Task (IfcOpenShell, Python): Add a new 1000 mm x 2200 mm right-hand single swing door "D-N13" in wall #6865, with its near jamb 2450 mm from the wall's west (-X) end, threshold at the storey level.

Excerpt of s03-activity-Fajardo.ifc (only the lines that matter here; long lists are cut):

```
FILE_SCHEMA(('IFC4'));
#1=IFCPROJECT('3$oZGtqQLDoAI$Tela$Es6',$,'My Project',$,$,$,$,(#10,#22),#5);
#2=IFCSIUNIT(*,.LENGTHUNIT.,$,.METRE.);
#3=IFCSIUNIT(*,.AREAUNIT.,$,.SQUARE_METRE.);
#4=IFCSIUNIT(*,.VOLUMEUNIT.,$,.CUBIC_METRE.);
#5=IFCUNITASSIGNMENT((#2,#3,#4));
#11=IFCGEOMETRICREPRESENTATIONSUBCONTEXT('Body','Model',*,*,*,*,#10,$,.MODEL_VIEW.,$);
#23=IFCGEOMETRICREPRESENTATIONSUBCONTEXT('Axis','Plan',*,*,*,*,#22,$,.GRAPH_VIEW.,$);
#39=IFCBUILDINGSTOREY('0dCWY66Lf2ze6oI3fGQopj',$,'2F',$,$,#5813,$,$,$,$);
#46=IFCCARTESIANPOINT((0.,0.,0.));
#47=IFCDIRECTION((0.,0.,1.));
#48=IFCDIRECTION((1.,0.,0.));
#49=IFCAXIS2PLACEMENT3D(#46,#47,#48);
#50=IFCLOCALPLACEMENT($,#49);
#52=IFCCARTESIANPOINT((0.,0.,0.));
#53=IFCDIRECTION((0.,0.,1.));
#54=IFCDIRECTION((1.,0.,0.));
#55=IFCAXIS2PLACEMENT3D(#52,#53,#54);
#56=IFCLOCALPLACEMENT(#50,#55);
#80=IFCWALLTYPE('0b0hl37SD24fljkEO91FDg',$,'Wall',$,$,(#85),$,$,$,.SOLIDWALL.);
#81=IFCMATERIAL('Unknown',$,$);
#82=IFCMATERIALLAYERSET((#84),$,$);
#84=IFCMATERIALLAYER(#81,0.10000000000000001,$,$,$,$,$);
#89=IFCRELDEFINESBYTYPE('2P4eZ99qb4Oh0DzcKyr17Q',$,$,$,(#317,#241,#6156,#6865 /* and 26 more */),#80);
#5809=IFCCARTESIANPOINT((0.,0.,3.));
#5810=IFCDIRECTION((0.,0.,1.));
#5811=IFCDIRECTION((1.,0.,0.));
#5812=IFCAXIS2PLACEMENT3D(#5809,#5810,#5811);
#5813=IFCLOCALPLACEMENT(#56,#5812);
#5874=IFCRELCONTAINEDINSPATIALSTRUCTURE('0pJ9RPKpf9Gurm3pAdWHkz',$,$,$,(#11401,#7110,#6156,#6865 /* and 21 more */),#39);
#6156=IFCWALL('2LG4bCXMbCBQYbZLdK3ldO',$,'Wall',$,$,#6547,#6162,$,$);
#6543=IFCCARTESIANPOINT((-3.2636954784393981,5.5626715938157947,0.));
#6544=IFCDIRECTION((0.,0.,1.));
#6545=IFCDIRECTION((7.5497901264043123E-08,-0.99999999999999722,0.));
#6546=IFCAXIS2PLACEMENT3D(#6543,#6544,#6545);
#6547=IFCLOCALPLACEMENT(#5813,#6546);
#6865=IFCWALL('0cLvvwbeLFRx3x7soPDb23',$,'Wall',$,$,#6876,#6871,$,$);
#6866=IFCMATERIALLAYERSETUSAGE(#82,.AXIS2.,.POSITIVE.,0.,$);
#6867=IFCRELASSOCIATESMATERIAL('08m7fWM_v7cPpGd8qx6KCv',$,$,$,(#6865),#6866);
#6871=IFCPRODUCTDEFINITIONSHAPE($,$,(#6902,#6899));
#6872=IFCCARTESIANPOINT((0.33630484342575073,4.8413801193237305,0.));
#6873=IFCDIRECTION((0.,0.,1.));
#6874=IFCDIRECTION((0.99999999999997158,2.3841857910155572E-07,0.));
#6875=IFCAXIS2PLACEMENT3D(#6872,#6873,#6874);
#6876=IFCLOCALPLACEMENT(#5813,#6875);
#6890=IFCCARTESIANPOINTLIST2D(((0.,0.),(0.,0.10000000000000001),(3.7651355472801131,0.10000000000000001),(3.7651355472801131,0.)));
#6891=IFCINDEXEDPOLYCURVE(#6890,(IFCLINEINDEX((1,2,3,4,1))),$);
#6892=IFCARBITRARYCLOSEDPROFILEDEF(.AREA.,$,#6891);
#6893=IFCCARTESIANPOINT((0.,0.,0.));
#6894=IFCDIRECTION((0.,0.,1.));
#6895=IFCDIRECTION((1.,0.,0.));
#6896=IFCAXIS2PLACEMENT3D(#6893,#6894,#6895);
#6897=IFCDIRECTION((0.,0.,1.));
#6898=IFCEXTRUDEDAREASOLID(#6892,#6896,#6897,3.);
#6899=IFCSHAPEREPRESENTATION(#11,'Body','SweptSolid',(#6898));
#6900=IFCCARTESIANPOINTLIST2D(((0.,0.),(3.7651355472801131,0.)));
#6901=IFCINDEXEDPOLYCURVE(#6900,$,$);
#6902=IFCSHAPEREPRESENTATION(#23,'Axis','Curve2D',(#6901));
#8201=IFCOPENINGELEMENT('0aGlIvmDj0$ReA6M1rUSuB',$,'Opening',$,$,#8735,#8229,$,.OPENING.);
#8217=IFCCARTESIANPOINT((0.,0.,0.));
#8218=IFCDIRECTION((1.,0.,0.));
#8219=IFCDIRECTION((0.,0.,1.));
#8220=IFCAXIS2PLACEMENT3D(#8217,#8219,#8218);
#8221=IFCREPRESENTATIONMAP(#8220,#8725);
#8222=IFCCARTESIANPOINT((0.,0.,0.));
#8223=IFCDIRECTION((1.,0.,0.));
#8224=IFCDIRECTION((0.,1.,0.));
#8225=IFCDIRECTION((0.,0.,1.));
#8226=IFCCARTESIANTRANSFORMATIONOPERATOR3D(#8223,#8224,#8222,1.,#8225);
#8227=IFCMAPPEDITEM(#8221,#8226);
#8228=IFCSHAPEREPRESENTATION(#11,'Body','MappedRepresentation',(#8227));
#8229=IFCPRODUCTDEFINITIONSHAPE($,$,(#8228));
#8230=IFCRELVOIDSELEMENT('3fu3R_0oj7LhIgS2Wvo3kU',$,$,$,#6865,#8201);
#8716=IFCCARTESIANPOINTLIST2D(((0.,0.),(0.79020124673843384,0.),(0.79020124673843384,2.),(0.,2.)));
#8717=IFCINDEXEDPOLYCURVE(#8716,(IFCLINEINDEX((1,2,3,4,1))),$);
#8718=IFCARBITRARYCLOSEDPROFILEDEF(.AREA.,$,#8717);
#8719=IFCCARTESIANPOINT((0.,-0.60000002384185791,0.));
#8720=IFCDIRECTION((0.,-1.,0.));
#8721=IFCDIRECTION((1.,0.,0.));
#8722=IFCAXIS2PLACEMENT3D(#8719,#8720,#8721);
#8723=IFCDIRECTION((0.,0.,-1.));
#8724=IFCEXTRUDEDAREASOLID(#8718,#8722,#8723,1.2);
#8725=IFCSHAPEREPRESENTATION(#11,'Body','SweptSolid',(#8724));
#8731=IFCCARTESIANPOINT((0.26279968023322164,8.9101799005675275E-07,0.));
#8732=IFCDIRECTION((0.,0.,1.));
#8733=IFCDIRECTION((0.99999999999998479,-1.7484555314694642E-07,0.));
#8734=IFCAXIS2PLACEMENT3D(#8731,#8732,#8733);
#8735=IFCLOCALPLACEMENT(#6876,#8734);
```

```python
import numpy as np
import ifcopenshell
import ifcopenshell.api.feature
import ifcopenshell.api.geometry
import ifcopenshell.api.root
import ifcopenshell.api.spatial
import ifcopenshell.geom
import ifcopenshell.util.element
import ifcopenshell.util.placement
import ifcopenshell.util.representation
import ifcopenshell.util.shape
import ifcopenshell.util.unit

model = ifcopenshell.open("s03-activity-Fajardo.ifc")
unit_scale = ifcopenshell.util.unit.calculate_unit_scale(model)
settings = ifcopenshell.geom.settings()


def volume(element):
    """Net volume in cubic metres, openings subtracted."""
    shape = ifcopenshell.geom.create_shape(settings, element)
    return ifcopenshell.util.shape.get_volume(shape.geometry)


wall = model.by_guid("0cLvvwbeLFRx3x7soPDb23")
storey = ifcopenshell.util.element.get_container(wall, ifc_class="IfcBuildingStorey")
context = ifcopenshell.util.representation.get_context(model, "Model", "Body", "MODEL_VIEW")
before = volume(wall)

width, height, from_end, sill = 1, 2.2, 2.45, 0.0  # metres

# The wall runs along its own X axis, and the end named is its -X end.
wall_shape = ifcopenshell.geom.create_shape(settings, wall)
x, y, z = ifcopenshell.util.shape.get_vertices(wall_shape.geometry).T
start = x.min() + from_end
face, thickness = float(y.min()), float(y.max() - y.min())
wall_matrix = ifcopenshell.util.placement.get_local_placement(wall.ObjectPlacement)
level = ifcopenshell.util.placement.get_local_placement(storey.ObjectPlacement)[2, 3]


def in_wall(x, y):
    """Placement at x, y metres in the wall's axes, at sill height."""
    matrix = wall_matrix.copy()
    matrix[:, 3] = wall_matrix @ np.array([x / unit_scale, y / unit_scale, 0.0, 1.0])
    matrix[2, 3] = level + sill / unit_scale
    return matrix


# Opening: a box that overshoots both wall faces by 50 mm.
opening = ifcopenshell.api.root.create_entity(model, ifc_class="IfcOpeningElement", predefined_type="OPENING")
box = ifcopenshell.api.geometry.add_wall_representation(
    model, context=context, length=width, height=height, thickness=thickness + 0.1
)
ifcopenshell.api.geometry.assign_representation(model, product=opening, representation=box)
ifcopenshell.api.geometry.edit_object_placement(model, product=opening, matrix=in_wall(start, face - 0.05), is_si=False)
ifcopenshell.api.feature.add_feature(model, feature=opening, element=wall)

door = ifcopenshell.api.root.create_entity(model, ifc_class="IfcDoor", name="D-N13", predefined_type="DOOR")
door.OverallWidth, door.OverallHeight = width / unit_scale, height / unit_scale
door.OperationType = "SINGLE_SWING_RIGHT"
body = ifcopenshell.api.geometry.add_door_representation(
    model,
    context=context,
    overall_width=door.OverallWidth,
    overall_height=door.OverallHeight,
    operation_type="SINGLE_SWING_RIGHT",
    lining_properties={"LiningDepth": thickness / unit_scale, "ThresholdDepth": thickness / unit_scale},
)
ifcopenshell.api.geometry.assign_representation(model, product=door, representation=body)
ifcopenshell.api.spatial.assign_container(model, products=[door], relating_structure=storey)
ifcopenshell.api.feature.add_filling(model, opening=opening, element=door)

# The lining spans the wall, so the door starts at the wall face.
ifcopenshell.api.geometry.edit_object_placement(model, product=door, matrix=in_wall(start, face), is_si=False)

after = volume(wall)

print(f"wall volume {before:.3f} -> {after:.3f} m3")

model.write("s03-activity-Fajardo_edited.ifc")
```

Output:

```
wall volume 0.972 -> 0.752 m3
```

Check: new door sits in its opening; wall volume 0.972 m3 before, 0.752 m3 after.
